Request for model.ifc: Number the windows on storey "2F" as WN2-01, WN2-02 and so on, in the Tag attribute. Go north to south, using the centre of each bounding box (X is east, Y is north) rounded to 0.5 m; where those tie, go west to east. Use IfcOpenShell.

First a look at what the model holds.

```python
import ifcopenshell
import ifcopenshell.util.element
import ifcopenshell.util.placement

model = ifcopenshell.open("model.ifc")
print(model.schema)
storey = next(s for s in model.by_type("IfcBuildingStorey") if s.Name == "2F")
windows = [e for e in ifcopenshell.util.element.get_decomposition(storey) if e.is_a("IfcWindow")]
for e in sorted(windows, key=lambda e: e.id()):
    origin = ifcopenshell.util.placement.get_local_placement(e.ObjectPlacement)[:3, 3]
    print(e.id(), e.Tag, e.Name, origin.round(2) + 0.0, sep=" | ")
```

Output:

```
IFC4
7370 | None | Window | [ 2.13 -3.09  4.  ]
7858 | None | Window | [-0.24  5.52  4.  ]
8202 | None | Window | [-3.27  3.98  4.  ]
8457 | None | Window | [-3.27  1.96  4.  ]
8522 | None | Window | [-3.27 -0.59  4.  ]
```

```python
import ifcopenshell
import ifcopenshell.geom
import ifcopenshell.util.element
import ifcopenshell.util.shape

model = ifcopenshell.open("model.ifc")
settings = ifcopenshell.geom.settings()
settings.set("use-world-coords", True)


def centre(element):
    shape = ifcopenshell.geom.create_shape(settings, element)
    return ifcopenshell.util.shape.get_bbox_centroid(shape.geometry)


storey = next(s for s in model.by_type("IfcBuildingStorey") if s.Name == "2F")
windows = [e for e in ifcopenshell.util.element.get_decomposition(storey) if e.is_a("IfcWindow")]

# Insertion points can sit at a corner or the storey origin, so sort by the geometry (in metres).
centres = {e: centre(e) for e in windows}
windows.sort(key=lambda e: (-round(centres[e][1] / 0.5), centres[e][0]))

for i, e in enumerate(windows, start=1):
    number = f"WN2-{i:02d}"
    e.Tag = number
    print(e.id(), number)

model.write("model-out.ifc")
```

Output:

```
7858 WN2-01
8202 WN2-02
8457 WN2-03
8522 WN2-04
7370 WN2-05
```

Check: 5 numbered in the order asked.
